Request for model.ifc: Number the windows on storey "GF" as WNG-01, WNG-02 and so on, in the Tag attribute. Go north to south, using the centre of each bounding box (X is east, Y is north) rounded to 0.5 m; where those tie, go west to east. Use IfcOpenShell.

First a look at what the model holds.

```python
import ifcopenshell
import ifcopenshell.util.element
import ifcopenshell.util.placement

model = ifcopenshell.open("model.ifc")
print(model.schema)
storey = next(s for s in model.by_type("IfcBuildingStorey") if s.Name == "GF")
windows = [e for e in ifcopenshell.util.element.get_decomposition(storey) if e.is_a("IfcWindow")]
for e in sorted(windows, key=lambda e: e.id()):
    origin = ifcopenshell.util.placement.get_local_placement(e.ObjectPlacement)[:3, 3]
    print(e.id(), e.Tag, e.Name, origin.round(2) + 0.0, sep=" | ")
```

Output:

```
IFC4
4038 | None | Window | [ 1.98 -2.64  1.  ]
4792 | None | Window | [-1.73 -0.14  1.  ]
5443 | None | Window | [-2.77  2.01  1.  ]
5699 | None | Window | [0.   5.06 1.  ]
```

```python
import ifcopenshell
import ifcopenshell.geom
import ifcopenshell.util.element
import ifcopenshell.util.shape

model = ifcopenshell.open("model.ifc")
settings = ifcopenshell.geom.settings()
settings.set("use-world-coords", True)


def centre(element):
    shape = ifcopenshell.geom.create_shape(settings, element)
    return ifcopenshell.util.shape.get_bbox_centroid(shape.geometry)


storey = next(s for s in model.by_type("IfcBuildingStorey") if s.Name == "GF")
windows = [e for e in ifcopenshell.util.element.get_decomposition(storey) if e.is_a("IfcWindow")]

# Insertion points can sit at a corner or the storey origin, so sort by the geometry (in metres).
centres = {e: centre(e) for e in windows}
windows.sort(key=lambda e: (-round(centres[e][1] / 0.5), centres[e][0]))

for i, e in enumerate(windows, start=1):
    number = f"WNG-{i:02d}"
    e.Tag = number
    print(e.id(), number)

model.write("model_edited.ifc")
```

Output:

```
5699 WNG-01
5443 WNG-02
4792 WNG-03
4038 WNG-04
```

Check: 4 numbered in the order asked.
